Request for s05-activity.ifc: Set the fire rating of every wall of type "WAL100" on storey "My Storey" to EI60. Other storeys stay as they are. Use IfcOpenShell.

First a look at what the model holds.

```python
import ifcopenshell
import ifcopenshell.util.element

model = ifcopenshell.open("s05-activity.ifc")
print(model.schema)
storey = next(s for s in model.by_type("IfcBuildingStorey") if s.Name == "My Storey")
walls = [e for e in ifcopenshell.util.element.get_decomposition(storey) if e.is_a("IfcWall")]
seen = {}
for e in walls:
    element_type = ifcopenshell.util.element.get_type(e)
    key = (element_type.Name if element_type != e and element_type else None, ifcopenshell.util.element.get_pset(e, "Pset_WallCommon", "FireRating"))
    seen[key] = seen.get(key, 0) + 1
for (name, value), count in sorted(seen.items(), key=str):
    print(count, "x", name, "|", value)
```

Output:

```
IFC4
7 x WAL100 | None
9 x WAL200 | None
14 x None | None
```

```python
import ifcopenshell
import ifcopenshell.api.pset
import ifcopenshell.util.element

model = ifcopenshell.open("s05-activity.ifc")

storey = next(s for s in model.by_type("IfcBuildingStorey") if s.Name == "My Storey")
walls = [e for e in ifcopenshell.util.element.get_decomposition(storey) if e.is_a("IfcWall")]

count = 0
for e in walls:
    element_type = ifcopenshell.util.element.get_type(e)
    if element_type in (None, e) or element_type.Name != "WAL100":
        continue
    # add_pset returns the element's existing set when there is one.
    pset = ifcopenshell.api.pset.add_pset(model, product=e, name="Pset_WallCommon")
    ifcopenshell.api.pset.edit_pset(model, pset=pset, properties={"FireRating": "EI60"})
    count += 1

print(count, "walls updated")

model.write("s05-activity_v2.ifc")
```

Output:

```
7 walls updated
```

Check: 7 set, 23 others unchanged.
